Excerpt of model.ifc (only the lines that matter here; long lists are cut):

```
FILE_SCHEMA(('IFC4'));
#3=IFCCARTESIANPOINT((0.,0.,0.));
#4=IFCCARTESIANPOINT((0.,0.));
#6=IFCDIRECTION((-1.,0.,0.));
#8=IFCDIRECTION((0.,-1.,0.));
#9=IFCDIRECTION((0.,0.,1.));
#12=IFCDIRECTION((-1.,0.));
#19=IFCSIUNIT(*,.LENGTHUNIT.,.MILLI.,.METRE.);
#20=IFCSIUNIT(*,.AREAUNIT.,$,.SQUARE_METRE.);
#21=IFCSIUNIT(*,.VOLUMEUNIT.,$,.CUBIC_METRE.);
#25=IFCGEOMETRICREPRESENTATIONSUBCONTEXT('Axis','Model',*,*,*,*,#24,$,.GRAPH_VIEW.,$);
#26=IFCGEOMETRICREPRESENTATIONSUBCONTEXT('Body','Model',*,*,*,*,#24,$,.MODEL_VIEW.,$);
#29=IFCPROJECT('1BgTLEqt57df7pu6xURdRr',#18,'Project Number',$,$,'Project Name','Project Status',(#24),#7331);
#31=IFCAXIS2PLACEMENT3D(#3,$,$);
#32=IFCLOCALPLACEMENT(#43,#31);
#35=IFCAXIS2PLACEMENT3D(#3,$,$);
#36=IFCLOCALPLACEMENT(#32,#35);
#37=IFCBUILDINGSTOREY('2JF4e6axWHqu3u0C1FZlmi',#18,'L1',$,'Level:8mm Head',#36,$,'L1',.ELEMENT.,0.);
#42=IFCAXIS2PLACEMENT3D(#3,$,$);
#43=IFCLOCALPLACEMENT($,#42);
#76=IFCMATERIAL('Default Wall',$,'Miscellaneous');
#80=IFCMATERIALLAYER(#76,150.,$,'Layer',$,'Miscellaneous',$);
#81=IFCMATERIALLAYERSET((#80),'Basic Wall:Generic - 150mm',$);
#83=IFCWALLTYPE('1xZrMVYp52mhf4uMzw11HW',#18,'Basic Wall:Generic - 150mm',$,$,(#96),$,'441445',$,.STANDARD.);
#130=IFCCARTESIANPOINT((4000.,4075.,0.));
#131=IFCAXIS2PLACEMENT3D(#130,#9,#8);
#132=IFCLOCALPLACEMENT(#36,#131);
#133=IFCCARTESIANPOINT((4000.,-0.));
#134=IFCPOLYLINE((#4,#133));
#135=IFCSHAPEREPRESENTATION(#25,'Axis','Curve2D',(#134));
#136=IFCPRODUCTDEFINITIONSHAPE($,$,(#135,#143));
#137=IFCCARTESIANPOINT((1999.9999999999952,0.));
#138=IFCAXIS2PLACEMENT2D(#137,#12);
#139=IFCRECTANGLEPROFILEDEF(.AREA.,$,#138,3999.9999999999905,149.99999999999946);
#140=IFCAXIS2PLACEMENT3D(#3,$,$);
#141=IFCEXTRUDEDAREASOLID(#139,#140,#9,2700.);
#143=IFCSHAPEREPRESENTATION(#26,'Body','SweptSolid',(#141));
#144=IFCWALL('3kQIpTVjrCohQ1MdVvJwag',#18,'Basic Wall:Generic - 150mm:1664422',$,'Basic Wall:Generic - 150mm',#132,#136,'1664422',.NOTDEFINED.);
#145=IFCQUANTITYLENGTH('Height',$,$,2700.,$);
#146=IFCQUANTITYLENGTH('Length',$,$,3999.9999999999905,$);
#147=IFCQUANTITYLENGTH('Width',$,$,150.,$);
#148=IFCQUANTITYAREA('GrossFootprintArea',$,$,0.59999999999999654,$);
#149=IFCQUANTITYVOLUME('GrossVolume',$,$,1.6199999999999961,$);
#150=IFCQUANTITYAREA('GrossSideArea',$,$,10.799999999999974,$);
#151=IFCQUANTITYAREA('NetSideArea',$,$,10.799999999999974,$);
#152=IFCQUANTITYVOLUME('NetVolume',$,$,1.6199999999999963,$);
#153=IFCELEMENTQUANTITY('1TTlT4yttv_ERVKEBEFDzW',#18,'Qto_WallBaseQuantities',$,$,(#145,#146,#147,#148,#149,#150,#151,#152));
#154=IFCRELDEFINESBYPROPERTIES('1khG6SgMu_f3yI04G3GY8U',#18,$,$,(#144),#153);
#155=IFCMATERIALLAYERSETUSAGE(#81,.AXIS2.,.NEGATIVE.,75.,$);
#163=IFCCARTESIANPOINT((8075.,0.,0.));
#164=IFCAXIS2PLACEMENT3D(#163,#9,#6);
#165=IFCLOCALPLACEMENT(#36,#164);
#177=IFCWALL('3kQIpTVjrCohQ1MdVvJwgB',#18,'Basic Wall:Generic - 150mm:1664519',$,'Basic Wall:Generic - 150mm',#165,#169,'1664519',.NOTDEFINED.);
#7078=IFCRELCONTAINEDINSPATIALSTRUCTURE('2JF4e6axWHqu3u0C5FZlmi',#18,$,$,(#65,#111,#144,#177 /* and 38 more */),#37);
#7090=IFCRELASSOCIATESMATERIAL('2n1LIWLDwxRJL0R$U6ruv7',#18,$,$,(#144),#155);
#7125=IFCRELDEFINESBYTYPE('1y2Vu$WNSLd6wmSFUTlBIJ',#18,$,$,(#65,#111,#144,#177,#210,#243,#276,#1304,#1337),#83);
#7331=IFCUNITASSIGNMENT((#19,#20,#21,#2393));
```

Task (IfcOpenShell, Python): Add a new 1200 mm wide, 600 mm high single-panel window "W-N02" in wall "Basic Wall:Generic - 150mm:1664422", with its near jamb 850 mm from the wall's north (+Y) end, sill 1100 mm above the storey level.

```python
import numpy as np
import ifcopenshell
import ifcopenshell.api.feature
import ifcopenshell.api.geometry
import ifcopenshell.api.pset
import ifcopenshell.api.root
import ifcopenshell.api.spatial
import ifcopenshell.geom
import ifcopenshell.util.element
import ifcopenshell.util.placement
import ifcopenshell.util.representation
import ifcopenshell.util.shape
import ifcopenshell.util.unit

model = ifcopenshell.open("model.ifc")
unit_scale = ifcopenshell.util.unit.calculate_unit_scale(model)
area_scale = ifcopenshell.util.unit.calculate_unit_scale(model, "AREAUNIT")
volume_scale = ifcopenshell.util.unit.calculate_unit_scale(model, "VOLUMEUNIT")
settings = ifcopenshell.geom.settings()


def volume(element):
    """Net volume in cubic metres, openings subtracted."""
    shape = ifcopenshell.geom.create_shape(settings, element)
    return ifcopenshell.util.shape.get_volume(shape.geometry)


wall = model.by_id(144)
storey = ifcopenshell.util.element.get_container(wall, ifc_class="IfcBuildingStorey")
context = ifcopenshell.util.representation.get_context(model, "Model", "Body", "MODEL_VIEW")
before = volume(wall)

width, height, from_end, sill = 1.2, 0.6, 0.85, 1.1  # metres

# The wall runs along its own X axis, and the end named is its -X end.
wall_shape = ifcopenshell.geom.create_shape(settings, wall)
x, y, z = ifcopenshell.util.shape.get_vertices(wall_shape.geometry).T
start = x.min() + from_end
face, thickness = float(y.min()), float(y.max() - y.min())
wall_matrix = ifcopenshell.util.placement.get_local_placement(wall.ObjectPlacement)
level = ifcopenshell.util.placement.get_local_placement(storey.ObjectPlacement)[2, 3]


def in_wall(x, y):
    """Placement at x, y metres in the wall's axes, at sill height."""
    matrix = wall_matrix.copy()
    matrix[:, 3] = wall_matrix @ np.array([x / unit_scale, y / unit_scale, 0.0, 1.0])
    matrix[2, 3] = level + sill / unit_scale
    return matrix


# Opening: a box that overshoots both wall faces by 50 mm.
opening = ifcopenshell.api.root.create_entity(model, ifc_class="IfcOpeningElement", predefined_type="OPENING")
box = ifcopenshell.api.geometry.add_wall_representation(
    model, context=context, length=width, height=height, thickness=thickness + 0.1
)
ifcopenshell.api.geometry.assign_representation(model, product=opening, representation=box)
ifcopenshell.api.geometry.edit_object_placement(model, product=opening, matrix=in_wall(start, face - 0.05), is_si=False)
ifcopenshell.api.feature.add_feature(model, feature=opening, element=wall)

window = ifcopenshell.api.root.create_entity(model, ifc_class="IfcWindow", name="W-N02", predefined_type="WINDOW")
window.OverallWidth, window.OverallHeight = width / unit_scale, height / unit_scale
window.PartitioningType = "SINGLE_PANEL"
body = ifcopenshell.api.geometry.add_window_representation(
    model,
    context=context,
    overall_width=window.OverallWidth,
    overall_height=window.OverallHeight,
    partition_type="SINGLE_PANEL",
)
ifcopenshell.api.geometry.assign_representation(model, product=window, representation=body)
ifcopenshell.api.spatial.assign_container(model, products=[window], relating_structure=storey)
ifcopenshell.api.feature.add_filling(model, opening=opening, element=window)

# Centre the window in the wall's thickness.
ifcopenshell.api.geometry.edit_object_placement(model, product=window, matrix=in_wall(start, face), is_si=False)
window_shape = ifcopenshell.geom.create_shape(settings, window)
depth = ifcopenshell.util.shape.get_vertices(window_shape.geometry)[:, 1]
offset = face + thickness / 2 - (depth.min() + depth.max()) / 2
ifcopenshell.api.geometry.edit_object_placement(model, product=window, matrix=in_wall(start, offset), is_si=False)

after = volume(wall)

# Update the wall's stored quantities.
qto = model.by_id(ifcopenshell.util.element.get_pset(wall, "Qto_WallBaseQuantities", should_inherit=False)["id"])
ifcopenshell.api.pset.edit_qto(model, qto=qto, properties={
    "NetSideArea": after / thickness / area_scale,
    "NetVolume": after / volume_scale,
})

print(f"wall volume {before:.3f} -> {after:.3f} m3")

model.write("model_updated.ifc")
```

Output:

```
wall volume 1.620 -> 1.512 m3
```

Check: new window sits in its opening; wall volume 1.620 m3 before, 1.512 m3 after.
